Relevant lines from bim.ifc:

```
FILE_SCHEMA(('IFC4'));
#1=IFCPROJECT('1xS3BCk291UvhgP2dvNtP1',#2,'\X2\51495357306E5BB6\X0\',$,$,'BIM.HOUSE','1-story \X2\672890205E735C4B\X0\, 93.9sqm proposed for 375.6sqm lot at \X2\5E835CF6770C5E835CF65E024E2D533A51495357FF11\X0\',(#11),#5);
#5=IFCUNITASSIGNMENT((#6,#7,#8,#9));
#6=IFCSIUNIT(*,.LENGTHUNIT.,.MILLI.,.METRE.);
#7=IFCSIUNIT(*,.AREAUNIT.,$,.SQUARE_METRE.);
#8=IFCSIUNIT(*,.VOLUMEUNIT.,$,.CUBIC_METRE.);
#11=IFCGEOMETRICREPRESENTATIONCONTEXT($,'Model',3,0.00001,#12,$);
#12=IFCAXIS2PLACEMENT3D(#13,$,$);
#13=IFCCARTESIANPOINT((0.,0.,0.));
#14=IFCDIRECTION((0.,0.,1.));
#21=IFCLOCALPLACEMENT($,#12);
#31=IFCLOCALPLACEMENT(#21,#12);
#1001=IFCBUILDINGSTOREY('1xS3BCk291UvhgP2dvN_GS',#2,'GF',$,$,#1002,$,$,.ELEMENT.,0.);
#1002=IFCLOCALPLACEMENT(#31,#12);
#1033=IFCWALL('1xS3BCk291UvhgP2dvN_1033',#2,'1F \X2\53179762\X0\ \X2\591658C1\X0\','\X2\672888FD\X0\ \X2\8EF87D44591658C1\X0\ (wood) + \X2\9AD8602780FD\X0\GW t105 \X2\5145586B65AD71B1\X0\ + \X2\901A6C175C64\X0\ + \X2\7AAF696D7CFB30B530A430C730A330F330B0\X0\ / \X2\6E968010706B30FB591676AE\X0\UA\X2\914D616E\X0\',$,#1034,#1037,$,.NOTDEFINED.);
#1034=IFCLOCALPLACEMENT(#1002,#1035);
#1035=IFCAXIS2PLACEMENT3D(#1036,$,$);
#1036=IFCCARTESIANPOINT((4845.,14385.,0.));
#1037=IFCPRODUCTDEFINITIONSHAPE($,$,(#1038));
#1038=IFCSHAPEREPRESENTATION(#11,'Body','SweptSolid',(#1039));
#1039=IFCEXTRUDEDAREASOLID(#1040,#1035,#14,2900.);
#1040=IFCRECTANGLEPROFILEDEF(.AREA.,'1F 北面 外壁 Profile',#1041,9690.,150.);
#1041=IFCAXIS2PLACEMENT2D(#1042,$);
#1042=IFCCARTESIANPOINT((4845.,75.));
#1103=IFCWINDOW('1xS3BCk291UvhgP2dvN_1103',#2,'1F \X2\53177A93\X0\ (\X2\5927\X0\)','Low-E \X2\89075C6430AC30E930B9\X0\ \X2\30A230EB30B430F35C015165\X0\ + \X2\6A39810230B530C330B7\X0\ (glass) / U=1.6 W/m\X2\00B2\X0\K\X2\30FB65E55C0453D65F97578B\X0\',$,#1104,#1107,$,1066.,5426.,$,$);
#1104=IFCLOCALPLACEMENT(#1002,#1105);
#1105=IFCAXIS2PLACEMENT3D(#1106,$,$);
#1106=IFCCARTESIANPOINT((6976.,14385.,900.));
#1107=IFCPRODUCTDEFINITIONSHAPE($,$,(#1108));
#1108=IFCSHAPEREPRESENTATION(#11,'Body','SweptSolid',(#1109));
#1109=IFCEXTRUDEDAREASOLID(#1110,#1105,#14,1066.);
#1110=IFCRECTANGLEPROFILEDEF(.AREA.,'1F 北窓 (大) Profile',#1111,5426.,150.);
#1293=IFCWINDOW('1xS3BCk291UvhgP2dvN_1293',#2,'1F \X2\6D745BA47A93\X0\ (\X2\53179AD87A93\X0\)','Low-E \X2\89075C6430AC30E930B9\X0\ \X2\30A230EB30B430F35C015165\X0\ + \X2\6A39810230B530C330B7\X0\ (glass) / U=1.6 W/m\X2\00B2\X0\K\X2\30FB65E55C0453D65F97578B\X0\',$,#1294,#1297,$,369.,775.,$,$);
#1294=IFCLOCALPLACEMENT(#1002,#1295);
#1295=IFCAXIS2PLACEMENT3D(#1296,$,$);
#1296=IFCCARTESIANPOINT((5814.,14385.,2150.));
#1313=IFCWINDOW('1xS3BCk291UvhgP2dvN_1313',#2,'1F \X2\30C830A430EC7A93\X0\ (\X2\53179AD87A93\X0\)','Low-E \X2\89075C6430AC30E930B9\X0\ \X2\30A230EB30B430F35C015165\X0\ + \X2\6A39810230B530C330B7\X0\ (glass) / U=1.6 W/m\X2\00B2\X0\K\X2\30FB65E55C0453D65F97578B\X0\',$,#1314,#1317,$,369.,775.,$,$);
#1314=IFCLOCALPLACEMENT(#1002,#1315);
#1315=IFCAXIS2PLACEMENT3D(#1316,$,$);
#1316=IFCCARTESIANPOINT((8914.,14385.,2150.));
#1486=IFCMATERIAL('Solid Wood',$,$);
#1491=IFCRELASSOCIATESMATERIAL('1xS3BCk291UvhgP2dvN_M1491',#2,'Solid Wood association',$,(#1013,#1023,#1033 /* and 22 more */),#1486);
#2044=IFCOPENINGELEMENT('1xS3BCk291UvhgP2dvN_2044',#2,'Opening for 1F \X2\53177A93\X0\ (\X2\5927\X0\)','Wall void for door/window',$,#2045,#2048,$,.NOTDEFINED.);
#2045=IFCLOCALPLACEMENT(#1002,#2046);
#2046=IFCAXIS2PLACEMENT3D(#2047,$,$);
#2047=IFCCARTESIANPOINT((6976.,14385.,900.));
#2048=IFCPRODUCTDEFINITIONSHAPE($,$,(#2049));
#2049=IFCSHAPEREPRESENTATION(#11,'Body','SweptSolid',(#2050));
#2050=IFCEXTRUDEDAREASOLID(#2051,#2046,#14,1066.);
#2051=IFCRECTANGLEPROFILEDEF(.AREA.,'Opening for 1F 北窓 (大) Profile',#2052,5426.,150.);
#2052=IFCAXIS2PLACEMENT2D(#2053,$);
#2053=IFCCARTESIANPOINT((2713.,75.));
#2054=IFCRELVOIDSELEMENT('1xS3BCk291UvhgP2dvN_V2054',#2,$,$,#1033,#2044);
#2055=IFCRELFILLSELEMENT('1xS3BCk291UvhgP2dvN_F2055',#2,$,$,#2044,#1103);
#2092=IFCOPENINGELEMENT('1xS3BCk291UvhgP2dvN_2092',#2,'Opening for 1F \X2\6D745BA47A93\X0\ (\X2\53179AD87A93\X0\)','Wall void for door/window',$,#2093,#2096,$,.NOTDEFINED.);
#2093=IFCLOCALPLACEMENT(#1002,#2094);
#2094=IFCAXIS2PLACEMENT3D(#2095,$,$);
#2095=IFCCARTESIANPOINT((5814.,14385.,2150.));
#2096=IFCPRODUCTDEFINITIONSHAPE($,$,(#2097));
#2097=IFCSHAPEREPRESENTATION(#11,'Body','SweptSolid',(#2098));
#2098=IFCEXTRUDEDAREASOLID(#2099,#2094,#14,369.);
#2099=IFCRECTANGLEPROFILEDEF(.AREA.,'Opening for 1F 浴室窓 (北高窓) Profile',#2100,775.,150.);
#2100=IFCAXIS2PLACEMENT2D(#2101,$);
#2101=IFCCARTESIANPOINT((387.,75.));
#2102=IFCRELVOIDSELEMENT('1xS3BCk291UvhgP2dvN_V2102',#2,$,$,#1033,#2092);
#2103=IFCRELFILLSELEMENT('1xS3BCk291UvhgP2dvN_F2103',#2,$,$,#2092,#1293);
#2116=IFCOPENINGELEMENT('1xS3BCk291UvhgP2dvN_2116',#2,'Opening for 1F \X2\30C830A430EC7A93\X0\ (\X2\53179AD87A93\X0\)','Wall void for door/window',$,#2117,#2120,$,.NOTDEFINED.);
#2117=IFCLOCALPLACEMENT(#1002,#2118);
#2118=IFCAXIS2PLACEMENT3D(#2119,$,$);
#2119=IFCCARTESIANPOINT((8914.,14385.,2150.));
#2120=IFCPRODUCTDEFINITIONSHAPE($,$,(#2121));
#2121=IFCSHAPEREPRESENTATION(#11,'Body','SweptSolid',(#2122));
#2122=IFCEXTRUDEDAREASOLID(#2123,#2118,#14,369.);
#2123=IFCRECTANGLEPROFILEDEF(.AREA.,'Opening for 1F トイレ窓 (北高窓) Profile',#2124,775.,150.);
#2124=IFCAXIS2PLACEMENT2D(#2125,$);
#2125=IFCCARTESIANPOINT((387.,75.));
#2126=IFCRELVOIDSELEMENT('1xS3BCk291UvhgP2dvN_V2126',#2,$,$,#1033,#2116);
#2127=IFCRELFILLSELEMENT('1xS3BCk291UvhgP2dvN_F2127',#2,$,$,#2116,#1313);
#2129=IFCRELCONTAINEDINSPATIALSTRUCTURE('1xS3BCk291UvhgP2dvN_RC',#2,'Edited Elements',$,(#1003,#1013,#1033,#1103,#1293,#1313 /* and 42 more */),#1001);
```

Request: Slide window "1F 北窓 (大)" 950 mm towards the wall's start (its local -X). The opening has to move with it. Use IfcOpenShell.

```python
import ifcopenshell
import ifcopenshell.api.geometry
import ifcopenshell.util.placement
import ifcopenshell.util.unit

model = ifcopenshell.open("bim.ifc")
unit_scale = ifcopenshell.util.unit.calculate_unit_scale(model)

window = model.by_guid("1xS3BCk291UvhgP2dvN_1103")
opening = window.FillsVoids[0].RelatingOpeningElement
wall = opening.VoidsElements[0].RelatingBuildingElement

wall_matrix = ifcopenshell.util.placement.get_local_placement(wall.ObjectPlacement)
shift = wall_matrix[:3, 0] * -0.95 / unit_scale
before = ifcopenshell.util.placement.get_local_placement(window.ObjectPlacement)[:3, 3].copy()

# The window is not placed relative to its opening, so move both.
for product in (opening, window):
    matrix = ifcopenshell.util.placement.get_local_placement(product.ObjectPlacement)
    matrix[:3, 3] += shift
    ifcopenshell.api.geometry.edit_object_placement(model, product=product, matrix=matrix, is_si=False)

after = ifcopenshell.util.placement.get_local_placement(window.ObjectPlacement)[:3, 3]
print("window moved by", (after - before).round(3) + 0.0)

model.write("bim-out.ifc")
```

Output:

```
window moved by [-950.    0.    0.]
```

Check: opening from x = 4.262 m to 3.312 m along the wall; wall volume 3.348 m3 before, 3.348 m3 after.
